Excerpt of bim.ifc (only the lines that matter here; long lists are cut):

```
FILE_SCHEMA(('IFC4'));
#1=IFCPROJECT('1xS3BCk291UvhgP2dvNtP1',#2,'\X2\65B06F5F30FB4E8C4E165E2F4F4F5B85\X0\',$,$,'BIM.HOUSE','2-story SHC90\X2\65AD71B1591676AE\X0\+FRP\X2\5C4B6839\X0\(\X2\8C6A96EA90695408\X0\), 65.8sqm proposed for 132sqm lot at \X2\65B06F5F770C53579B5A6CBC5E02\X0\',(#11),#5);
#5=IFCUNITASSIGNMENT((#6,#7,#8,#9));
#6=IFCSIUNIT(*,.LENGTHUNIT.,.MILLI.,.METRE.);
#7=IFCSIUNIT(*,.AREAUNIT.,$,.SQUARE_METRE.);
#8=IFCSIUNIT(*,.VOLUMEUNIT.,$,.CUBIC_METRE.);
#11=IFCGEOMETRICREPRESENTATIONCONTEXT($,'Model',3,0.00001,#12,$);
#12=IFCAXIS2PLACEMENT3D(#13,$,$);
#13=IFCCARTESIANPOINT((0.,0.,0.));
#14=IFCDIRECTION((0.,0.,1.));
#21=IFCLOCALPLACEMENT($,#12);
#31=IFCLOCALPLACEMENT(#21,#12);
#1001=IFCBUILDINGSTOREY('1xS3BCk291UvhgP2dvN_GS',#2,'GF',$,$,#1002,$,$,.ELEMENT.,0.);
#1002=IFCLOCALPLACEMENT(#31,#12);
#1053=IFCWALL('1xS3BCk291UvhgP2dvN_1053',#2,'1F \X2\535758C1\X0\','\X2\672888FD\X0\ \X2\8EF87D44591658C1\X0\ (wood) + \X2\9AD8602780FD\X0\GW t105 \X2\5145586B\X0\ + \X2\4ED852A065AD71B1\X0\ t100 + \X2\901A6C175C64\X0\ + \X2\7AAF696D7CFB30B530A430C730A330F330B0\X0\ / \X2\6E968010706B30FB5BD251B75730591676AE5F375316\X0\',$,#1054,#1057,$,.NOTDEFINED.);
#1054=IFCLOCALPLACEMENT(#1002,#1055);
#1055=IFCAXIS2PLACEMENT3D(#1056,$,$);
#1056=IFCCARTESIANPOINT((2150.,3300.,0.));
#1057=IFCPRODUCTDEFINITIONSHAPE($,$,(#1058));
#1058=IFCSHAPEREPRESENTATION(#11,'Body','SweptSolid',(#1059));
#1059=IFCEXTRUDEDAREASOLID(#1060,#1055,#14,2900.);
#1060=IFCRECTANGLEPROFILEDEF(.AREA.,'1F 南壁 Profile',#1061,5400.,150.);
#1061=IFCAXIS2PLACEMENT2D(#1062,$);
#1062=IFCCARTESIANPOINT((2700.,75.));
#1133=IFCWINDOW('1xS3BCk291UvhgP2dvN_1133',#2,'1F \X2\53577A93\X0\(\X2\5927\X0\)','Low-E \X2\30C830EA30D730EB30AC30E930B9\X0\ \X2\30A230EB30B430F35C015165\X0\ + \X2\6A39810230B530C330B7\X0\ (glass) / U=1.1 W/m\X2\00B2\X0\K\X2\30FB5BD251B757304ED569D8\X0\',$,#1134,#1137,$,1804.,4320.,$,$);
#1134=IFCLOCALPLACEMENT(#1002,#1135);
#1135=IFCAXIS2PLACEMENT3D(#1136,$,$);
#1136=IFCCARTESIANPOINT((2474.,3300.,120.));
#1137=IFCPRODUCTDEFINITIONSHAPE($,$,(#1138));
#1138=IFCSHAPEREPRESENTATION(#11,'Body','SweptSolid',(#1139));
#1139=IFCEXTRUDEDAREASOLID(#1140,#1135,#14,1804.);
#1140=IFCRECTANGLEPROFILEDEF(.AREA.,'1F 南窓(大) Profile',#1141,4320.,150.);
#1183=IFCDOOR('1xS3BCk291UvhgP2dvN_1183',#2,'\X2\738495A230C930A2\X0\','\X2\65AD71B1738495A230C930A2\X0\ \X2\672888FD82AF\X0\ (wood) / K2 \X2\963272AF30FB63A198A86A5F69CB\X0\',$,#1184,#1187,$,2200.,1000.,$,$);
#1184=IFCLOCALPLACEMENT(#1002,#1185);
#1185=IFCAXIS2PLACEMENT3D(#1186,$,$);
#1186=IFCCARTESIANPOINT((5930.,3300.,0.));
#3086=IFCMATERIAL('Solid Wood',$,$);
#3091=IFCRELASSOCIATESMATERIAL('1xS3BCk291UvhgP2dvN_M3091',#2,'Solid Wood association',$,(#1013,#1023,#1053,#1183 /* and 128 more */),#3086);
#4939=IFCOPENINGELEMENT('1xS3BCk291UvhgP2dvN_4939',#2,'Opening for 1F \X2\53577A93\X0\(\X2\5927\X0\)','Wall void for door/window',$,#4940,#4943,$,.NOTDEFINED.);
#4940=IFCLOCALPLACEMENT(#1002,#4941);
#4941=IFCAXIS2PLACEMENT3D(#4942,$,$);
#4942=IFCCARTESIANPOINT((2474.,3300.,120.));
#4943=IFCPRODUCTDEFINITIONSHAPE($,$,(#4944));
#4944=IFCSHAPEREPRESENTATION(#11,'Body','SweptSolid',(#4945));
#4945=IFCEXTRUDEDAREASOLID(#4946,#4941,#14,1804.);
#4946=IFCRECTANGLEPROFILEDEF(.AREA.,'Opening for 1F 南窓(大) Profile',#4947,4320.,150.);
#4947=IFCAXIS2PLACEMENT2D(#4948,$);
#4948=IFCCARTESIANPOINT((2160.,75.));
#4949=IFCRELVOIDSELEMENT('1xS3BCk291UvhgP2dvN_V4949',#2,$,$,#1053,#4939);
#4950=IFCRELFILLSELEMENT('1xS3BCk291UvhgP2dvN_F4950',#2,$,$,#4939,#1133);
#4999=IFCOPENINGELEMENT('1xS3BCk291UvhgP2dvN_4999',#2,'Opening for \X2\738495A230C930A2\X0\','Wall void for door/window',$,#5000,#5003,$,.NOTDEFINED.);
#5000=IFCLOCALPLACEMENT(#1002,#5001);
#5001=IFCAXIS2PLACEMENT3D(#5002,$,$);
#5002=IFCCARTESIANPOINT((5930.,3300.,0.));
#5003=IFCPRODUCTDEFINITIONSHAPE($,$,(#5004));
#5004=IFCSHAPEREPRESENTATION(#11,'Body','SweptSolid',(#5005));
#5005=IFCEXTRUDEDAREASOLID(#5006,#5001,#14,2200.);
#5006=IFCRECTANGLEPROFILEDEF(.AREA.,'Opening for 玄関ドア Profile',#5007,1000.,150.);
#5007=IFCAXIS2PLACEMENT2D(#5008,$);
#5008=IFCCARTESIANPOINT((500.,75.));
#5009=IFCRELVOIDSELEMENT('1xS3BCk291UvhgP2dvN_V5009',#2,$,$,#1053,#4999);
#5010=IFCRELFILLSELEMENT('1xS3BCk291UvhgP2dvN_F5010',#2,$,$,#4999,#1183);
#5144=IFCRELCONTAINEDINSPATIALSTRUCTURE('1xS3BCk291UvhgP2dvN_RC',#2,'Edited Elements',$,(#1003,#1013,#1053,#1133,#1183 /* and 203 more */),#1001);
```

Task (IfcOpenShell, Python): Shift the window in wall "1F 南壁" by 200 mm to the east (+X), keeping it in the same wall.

```python
import ifcopenshell
import ifcopenshell.api.geometry
import ifcopenshell.util.placement

model = ifcopenshell.open("bim.ifc")

window = model.by_guid("1xS3BCk291UvhgP2dvN_1133")
opening = window.FillsVoids[0].RelatingOpeningElement
wall = opening.VoidsElements[0].RelatingBuildingElement

wall_matrix = ifcopenshell.util.placement.get_local_placement(wall.ObjectPlacement)
shift = wall_matrix[:3, 0] * 200.0
before = ifcopenshell.util.placement.get_local_placement(window.ObjectPlacement)[:3, 3].copy()

# The window is not placed relative to its opening, so move both.
for product in (opening, window):
    matrix = ifcopenshell.util.placement.get_local_placement(product.ObjectPlacement)
    matrix[:3, 3] += shift
    ifcopenshell.api.geometry.edit_object_placement(model, product=product, matrix=matrix, is_si=False)

after = ifcopenshell.util.placement.get_local_placement(window.ObjectPlacement)[:3, 3]
print("window moved by", (after - before).round(3) + 0.0)

model.write("bim_rev.ifc")
```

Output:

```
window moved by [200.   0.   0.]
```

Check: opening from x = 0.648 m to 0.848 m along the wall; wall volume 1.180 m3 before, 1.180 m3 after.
